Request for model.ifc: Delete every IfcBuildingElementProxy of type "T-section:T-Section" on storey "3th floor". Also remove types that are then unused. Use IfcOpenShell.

First a look at what the model holds.

```python
import ifcopenshell
import ifcopenshell.util.element

model = ifcopenshell.open("model.ifc")
print(model.schema)
storey = next(s for s in model.by_type("IfcBuildingStorey") if s.Name == "3th floor")
proxies = [e for e in ifcopenshell.util.element.get_decomposition(storey) if e.is_a("IfcBuildingElementProxy")]
seen = {}
for e in proxies:
    element_type = ifcopenshell.util.element.get_type(e)
    name = element_type.Name if element_type not in (None, e) else None
    seen[name] = seen.get(name, 0) + 1
for name, count in sorted(seen.items(), key=str):
    print(count, "x", name)
```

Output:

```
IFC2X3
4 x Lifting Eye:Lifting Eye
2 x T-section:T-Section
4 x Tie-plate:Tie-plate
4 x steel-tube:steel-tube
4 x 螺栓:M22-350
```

```python
import ifcopenshell
import ifcopenshell.api.root
import ifcopenshell.util.element

model = ifcopenshell.open("model.ifc")

storey = next(s for s in model.by_type("IfcBuildingStorey") if s.Name == "3th floor")
proxies = [e for e in ifcopenshell.util.element.get_decomposition(storey) if e.is_a("IfcBuildingElementProxy")]
targets = [e for e in proxies if (t := ifcopenshell.util.element.get_type(e)) not in (None, e) and t.Name == "T-section:T-Section"]
types = {ifcopenshell.util.element.get_type(e) for e in targets} - {None, *targets}

for e in targets:
    ifcopenshell.api.root.remove_product(model, product=e)
print(len(targets), "removed")

unused = [t for t in types if not ifcopenshell.util.element.get_types(t)]
for t in unused:
    ifcopenshell.api.root.remove_product(model, product=t)
print(len(unused), "unused types removed")

model.write("model-out.ifc")
```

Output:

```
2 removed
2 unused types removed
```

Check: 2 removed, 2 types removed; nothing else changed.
